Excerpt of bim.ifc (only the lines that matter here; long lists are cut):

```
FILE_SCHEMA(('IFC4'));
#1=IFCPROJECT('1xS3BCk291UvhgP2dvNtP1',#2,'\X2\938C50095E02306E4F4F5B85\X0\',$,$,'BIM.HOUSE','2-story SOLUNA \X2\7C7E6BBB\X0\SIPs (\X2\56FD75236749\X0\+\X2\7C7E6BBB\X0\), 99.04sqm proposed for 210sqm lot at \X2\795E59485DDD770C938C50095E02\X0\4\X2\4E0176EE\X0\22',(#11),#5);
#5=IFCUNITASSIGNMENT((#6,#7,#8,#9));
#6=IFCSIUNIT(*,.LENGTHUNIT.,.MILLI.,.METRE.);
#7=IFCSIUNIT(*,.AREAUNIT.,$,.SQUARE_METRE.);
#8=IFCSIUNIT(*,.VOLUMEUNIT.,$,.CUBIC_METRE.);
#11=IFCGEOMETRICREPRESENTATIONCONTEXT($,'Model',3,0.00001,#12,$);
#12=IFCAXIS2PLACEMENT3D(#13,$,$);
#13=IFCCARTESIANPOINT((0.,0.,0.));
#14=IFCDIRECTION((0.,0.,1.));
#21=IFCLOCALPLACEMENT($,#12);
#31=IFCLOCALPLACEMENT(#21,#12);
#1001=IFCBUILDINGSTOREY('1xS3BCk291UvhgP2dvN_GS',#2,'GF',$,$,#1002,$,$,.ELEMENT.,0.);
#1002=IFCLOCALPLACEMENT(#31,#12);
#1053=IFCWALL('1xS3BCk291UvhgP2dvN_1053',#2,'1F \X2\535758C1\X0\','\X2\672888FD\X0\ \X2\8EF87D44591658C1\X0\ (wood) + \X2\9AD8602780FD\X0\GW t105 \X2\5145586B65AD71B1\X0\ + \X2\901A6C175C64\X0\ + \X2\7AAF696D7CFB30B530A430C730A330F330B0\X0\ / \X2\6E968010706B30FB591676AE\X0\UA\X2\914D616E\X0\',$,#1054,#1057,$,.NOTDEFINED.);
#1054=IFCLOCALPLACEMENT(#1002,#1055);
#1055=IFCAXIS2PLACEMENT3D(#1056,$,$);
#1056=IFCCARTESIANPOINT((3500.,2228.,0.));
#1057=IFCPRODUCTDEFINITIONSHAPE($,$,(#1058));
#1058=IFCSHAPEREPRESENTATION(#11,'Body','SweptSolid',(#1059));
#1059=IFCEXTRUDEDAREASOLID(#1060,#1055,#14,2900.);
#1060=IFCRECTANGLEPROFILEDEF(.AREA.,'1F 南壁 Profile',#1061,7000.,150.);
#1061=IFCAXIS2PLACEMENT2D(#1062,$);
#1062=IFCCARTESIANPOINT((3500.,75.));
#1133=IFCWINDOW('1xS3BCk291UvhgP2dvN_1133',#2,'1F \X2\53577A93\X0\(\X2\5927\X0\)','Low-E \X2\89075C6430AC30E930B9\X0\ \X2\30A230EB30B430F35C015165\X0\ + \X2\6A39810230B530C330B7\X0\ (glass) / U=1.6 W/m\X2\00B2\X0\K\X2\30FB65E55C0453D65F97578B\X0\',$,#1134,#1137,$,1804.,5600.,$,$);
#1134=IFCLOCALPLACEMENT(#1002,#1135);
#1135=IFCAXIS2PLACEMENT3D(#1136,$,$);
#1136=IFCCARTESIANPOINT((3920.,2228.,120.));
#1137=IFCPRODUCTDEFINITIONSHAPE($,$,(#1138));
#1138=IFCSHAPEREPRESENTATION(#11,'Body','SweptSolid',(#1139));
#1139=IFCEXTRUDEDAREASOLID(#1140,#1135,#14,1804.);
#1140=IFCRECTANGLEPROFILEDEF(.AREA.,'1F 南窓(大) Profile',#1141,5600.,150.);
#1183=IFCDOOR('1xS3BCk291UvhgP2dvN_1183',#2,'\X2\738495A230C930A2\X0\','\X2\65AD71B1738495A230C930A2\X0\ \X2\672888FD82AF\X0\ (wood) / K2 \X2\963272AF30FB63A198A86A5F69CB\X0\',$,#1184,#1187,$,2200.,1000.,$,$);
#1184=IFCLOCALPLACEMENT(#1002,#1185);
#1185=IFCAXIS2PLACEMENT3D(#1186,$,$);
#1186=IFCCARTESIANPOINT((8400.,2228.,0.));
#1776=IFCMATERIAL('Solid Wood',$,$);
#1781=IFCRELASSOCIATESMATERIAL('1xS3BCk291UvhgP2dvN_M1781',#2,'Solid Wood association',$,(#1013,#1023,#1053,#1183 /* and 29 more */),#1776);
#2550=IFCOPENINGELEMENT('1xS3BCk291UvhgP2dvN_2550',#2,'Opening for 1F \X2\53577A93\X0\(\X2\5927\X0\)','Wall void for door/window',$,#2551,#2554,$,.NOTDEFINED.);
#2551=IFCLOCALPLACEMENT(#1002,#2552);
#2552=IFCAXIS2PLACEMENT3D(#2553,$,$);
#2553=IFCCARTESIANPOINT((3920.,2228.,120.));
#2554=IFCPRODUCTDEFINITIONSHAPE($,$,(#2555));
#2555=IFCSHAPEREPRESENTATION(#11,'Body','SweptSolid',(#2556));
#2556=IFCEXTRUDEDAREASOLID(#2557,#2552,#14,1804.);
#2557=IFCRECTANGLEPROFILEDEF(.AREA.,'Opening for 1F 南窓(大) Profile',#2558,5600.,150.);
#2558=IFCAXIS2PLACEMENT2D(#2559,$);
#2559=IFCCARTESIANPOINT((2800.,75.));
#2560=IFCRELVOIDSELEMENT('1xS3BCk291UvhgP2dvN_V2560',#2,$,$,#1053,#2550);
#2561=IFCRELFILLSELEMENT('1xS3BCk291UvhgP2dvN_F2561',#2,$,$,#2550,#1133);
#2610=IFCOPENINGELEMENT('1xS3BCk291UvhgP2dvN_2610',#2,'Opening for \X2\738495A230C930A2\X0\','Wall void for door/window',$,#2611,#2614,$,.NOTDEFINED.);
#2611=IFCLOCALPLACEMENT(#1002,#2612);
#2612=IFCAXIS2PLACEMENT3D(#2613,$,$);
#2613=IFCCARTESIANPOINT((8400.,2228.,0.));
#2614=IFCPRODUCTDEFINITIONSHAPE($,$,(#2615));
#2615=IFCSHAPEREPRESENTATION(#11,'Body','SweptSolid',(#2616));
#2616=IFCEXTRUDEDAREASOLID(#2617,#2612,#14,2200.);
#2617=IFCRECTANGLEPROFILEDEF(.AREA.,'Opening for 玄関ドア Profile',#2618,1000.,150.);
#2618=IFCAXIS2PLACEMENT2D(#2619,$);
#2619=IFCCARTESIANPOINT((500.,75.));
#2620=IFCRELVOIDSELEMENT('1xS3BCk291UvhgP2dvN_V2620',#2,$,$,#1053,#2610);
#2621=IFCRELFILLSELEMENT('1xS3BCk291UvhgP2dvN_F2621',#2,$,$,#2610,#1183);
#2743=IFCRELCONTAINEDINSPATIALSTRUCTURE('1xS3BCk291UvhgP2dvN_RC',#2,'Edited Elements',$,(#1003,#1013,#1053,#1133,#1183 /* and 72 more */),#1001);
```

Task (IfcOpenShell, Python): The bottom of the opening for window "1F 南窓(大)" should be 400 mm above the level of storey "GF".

```python
import numpy as np
import ifcopenshell
import ifcopenshell.api.geometry
import ifcopenshell.geom
import ifcopenshell.util.element
import ifcopenshell.util.placement
import ifcopenshell.util.shape
import ifcopenshell.util.unit

model = ifcopenshell.open("bim.ifc")
unit_scale = ifcopenshell.util.unit.calculate_unit_scale(model)

window = model.by_guid("1xS3BCk291UvhgP2dvN_1133")
opening = window.FillsVoids[0].RelatingOpeningElement
storey = ifcopenshell.util.element.get_container(window, ifc_class="IfcBuildingStorey")
level = ifcopenshell.util.placement.get_local_placement(storey.ObjectPlacement)[2, 3]

# The opening's origin need not be at the sill, so measure its lowest point.
shape = ifcopenshell.geom.create_shape(ifcopenshell.geom.settings(), opening)
bottom = ifcopenshell.util.shape.get_shape_bottom_elevation(shape, shape.geometry) / unit_scale
dz = level + 0.4 / unit_scale - bottom

shift = np.array([0.0, 0.0, dz])
# The window is not placed relative to its opening, so move both.
for product in (opening, window):
    matrix = ifcopenshell.util.placement.get_local_placement(product.ObjectPlacement)
    matrix[:3, 3] += shift
    ifcopenshell.api.geometry.edit_object_placement(model, product=product, matrix=matrix, is_si=False)

print(f"moved by {dz * unit_scale:+.3f} m")

model.write("bim_v2.ifc")
```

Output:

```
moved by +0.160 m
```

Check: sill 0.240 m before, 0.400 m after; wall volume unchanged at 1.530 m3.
